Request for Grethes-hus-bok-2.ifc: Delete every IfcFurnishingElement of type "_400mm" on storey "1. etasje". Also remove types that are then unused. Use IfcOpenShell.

First a look at what the model holds.

```python
import ifcopenshell
import ifcopenshell.util.element

model = ifcopenshell.open("Grethes-hus-bok-2.ifc")
print(model.schema)
storey = next(s for s in model.by_type("IfcBuildingStorey") if s.Name == "1. etasje")
furniture = [e for e in ifcopenshell.util.element.get_decomposition(storey) if e.is_a("IfcFurnishingElement")]
seen = {}
for e in furniture:
    element_type = ifcopenshell.util.element.get_type(e)
    name = element_type.Name if element_type not in (None, e) else None
    seen[name] = seen.get(name, 0) + 1
for name, count in sorted(seen.items(), key=str):
    print(count, "x", name)
```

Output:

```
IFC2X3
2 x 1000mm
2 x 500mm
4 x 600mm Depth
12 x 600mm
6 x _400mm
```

```python
import ifcopenshell
import ifcopenshell.api.root
import ifcopenshell.util.element

model = ifcopenshell.open("Grethes-hus-bok-2.ifc")

storey = next(s for s in model.by_type("IfcBuildingStorey") if s.Name == "1. etasje")
furniture = [e for e in ifcopenshell.util.element.get_decomposition(storey) if e.is_a("IfcFurnishingElement")]
targets = [e for e in furniture if (t := ifcopenshell.util.element.get_type(e)) not in (None, e) and t.Name == "_400mm"]
types = {ifcopenshell.util.element.get_type(e) for e in targets} - {None, *targets}

for e in targets:
    ifcopenshell.api.root.remove_product(model, product=e)
print(len(targets), "removed")

unused = [t for t in types if not ifcopenshell.util.element.get_types(t)]
for t in unused:
    ifcopenshell.api.root.remove_product(model, product=t)
print(len(unused), "unused types removed")

model.write("Grethes-hus-bok-2_rev.ifc")
```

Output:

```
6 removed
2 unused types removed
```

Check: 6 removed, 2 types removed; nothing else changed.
